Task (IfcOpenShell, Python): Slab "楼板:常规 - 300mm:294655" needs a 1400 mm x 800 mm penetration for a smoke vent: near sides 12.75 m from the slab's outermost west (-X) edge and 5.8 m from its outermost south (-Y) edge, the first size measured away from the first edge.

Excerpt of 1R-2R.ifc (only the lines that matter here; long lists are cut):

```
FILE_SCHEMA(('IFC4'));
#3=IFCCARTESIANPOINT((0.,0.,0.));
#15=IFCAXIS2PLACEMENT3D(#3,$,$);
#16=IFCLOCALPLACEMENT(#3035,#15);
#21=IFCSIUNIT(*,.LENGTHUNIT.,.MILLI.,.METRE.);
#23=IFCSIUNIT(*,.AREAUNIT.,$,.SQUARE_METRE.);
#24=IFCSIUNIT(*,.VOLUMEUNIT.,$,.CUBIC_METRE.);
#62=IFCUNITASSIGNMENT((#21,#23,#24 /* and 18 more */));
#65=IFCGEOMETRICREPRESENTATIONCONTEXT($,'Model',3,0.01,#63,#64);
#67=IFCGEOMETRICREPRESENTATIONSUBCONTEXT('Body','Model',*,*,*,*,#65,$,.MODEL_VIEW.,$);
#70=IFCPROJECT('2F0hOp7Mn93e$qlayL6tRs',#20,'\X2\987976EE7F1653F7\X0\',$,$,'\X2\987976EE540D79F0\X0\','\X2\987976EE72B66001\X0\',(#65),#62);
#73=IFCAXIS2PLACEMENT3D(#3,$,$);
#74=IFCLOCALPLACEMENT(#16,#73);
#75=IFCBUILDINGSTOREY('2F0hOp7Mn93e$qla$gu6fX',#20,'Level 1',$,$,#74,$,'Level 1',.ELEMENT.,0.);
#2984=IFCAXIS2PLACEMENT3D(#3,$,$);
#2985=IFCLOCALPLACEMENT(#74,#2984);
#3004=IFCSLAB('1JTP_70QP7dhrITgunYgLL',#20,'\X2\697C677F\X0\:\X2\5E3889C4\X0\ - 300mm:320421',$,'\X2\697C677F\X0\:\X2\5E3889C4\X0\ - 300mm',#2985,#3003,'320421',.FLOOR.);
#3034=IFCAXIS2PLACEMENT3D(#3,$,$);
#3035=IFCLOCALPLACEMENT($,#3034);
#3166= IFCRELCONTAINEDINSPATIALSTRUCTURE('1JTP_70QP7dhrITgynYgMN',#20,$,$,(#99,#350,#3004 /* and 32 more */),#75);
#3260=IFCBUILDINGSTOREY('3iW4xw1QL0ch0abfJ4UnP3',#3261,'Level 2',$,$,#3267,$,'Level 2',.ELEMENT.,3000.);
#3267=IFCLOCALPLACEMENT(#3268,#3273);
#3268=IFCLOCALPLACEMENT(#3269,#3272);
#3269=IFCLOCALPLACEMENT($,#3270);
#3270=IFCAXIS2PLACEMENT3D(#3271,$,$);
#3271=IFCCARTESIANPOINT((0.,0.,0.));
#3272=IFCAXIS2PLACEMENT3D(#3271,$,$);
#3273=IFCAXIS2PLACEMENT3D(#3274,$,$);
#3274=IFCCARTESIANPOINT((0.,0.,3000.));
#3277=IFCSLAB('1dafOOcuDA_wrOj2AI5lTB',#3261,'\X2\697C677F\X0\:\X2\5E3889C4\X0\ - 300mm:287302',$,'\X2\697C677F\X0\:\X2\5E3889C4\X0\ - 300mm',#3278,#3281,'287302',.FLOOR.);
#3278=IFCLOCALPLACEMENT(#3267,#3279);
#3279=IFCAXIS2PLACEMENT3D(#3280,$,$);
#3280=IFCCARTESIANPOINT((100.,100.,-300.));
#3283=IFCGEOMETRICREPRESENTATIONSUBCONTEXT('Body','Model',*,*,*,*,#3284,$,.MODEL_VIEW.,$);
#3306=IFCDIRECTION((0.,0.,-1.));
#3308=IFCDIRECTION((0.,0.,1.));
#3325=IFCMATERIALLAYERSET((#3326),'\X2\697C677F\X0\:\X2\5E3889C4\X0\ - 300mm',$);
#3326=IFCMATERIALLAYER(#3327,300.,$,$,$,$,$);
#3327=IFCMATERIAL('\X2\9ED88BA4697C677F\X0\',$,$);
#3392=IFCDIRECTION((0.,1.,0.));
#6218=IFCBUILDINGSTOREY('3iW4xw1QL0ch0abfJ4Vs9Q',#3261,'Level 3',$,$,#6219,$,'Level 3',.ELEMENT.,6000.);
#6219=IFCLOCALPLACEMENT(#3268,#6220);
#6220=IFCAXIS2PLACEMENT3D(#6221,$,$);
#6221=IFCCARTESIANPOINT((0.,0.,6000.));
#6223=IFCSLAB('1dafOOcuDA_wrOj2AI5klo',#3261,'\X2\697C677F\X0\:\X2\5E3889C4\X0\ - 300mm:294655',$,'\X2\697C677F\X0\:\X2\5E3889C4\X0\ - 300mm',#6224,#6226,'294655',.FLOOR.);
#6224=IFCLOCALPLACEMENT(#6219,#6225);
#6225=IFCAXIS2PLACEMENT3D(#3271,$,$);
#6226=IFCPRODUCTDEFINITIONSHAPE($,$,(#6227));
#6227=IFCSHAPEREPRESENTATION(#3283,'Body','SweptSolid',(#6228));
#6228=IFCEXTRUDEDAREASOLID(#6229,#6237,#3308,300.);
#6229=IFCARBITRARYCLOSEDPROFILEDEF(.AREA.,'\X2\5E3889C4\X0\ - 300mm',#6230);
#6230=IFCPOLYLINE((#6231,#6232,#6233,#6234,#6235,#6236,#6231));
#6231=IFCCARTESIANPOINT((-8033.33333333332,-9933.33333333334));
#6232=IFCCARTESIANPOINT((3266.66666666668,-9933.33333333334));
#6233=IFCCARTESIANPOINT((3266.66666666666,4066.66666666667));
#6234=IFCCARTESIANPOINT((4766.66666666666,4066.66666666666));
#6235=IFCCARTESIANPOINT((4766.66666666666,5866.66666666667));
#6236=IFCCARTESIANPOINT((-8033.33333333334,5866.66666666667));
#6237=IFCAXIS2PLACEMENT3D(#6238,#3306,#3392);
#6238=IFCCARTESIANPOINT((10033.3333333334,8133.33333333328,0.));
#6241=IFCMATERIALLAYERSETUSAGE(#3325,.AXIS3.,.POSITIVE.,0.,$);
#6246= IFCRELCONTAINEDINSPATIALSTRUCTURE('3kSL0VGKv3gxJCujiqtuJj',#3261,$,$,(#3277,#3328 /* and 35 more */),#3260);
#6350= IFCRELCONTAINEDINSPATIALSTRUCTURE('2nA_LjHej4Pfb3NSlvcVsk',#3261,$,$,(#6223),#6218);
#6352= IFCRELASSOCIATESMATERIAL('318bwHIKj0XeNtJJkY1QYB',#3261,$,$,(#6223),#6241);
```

```python
import numpy as np
import ifcopenshell
import ifcopenshell.api.feature
import ifcopenshell.api.geometry
import ifcopenshell.api.root
import ifcopenshell.geom
import ifcopenshell.util.placement
import ifcopenshell.util.representation
import ifcopenshell.util.shape
import ifcopenshell.util.unit

model = ifcopenshell.open("1R-2R.ifc")
unit_scale = ifcopenshell.util.unit.calculate_unit_scale(model)
settings = ifcopenshell.geom.settings()


def volume(element):
    """Net volume in cubic metres, openings subtracted."""
    shape = ifcopenshell.geom.create_shape(settings, element)
    return ifcopenshell.util.shape.get_volume(shape.geometry)


slab = model.by_guid("1dafOOcuDA_wrOj2AI5klo")
before = volume(slab)

# Extent in the slab's own axes, in metres. The edges named are its -X and -Y sides.
slab_shape = ifcopenshell.geom.create_shape(settings, slab)
vertices = ifcopenshell.util.shape.get_vertices(slab_shape.geometry)
x_min, y_min, bottom = vertices.min(axis=0)
top = vertices[:, 2].max()

opening = ifcopenshell.api.root.create_entity(model, ifc_class="IfcOpeningElement", name="Smoke vent opening", predefined_type="OPENING")
context = ifcopenshell.util.representation.get_context(model, "Model", "Body", "MODEL_VIEW")
width, depth = 1.4, 0.8
outline = [(0.0, 0.0), (width, 0.0), (width, depth), (0.0, depth), (0.0, 0.0)]
# Overshoot both faces by 50 mm so the cut is clean.
shape = ifcopenshell.api.geometry.add_slab_representation(
    model, context=context, depth=top - bottom + 0.1, polyline=outline
)
ifcopenshell.api.geometry.assign_representation(model, product=opening, representation=shape)

matrix = ifcopenshell.util.placement.get_local_placement(slab.ObjectPlacement)
matrix[:, 3] = matrix @ np.append(np.array([x_min + 12.75, y_min + 5.8, bottom - 0.05]) / unit_scale, 1.0)
ifcopenshell.api.geometry.edit_object_placement(model, product=opening, matrix=matrix, is_si=False)
ifcopenshell.api.feature.add_feature(model, feature=opening, element=slab)

after = volume(slab)

print(f"slab volume {before:.3f} -> {after:.3f} m3")

model.write("1R-2R-out.ifc")
```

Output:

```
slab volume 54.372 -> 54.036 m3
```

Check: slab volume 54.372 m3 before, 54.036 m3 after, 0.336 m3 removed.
